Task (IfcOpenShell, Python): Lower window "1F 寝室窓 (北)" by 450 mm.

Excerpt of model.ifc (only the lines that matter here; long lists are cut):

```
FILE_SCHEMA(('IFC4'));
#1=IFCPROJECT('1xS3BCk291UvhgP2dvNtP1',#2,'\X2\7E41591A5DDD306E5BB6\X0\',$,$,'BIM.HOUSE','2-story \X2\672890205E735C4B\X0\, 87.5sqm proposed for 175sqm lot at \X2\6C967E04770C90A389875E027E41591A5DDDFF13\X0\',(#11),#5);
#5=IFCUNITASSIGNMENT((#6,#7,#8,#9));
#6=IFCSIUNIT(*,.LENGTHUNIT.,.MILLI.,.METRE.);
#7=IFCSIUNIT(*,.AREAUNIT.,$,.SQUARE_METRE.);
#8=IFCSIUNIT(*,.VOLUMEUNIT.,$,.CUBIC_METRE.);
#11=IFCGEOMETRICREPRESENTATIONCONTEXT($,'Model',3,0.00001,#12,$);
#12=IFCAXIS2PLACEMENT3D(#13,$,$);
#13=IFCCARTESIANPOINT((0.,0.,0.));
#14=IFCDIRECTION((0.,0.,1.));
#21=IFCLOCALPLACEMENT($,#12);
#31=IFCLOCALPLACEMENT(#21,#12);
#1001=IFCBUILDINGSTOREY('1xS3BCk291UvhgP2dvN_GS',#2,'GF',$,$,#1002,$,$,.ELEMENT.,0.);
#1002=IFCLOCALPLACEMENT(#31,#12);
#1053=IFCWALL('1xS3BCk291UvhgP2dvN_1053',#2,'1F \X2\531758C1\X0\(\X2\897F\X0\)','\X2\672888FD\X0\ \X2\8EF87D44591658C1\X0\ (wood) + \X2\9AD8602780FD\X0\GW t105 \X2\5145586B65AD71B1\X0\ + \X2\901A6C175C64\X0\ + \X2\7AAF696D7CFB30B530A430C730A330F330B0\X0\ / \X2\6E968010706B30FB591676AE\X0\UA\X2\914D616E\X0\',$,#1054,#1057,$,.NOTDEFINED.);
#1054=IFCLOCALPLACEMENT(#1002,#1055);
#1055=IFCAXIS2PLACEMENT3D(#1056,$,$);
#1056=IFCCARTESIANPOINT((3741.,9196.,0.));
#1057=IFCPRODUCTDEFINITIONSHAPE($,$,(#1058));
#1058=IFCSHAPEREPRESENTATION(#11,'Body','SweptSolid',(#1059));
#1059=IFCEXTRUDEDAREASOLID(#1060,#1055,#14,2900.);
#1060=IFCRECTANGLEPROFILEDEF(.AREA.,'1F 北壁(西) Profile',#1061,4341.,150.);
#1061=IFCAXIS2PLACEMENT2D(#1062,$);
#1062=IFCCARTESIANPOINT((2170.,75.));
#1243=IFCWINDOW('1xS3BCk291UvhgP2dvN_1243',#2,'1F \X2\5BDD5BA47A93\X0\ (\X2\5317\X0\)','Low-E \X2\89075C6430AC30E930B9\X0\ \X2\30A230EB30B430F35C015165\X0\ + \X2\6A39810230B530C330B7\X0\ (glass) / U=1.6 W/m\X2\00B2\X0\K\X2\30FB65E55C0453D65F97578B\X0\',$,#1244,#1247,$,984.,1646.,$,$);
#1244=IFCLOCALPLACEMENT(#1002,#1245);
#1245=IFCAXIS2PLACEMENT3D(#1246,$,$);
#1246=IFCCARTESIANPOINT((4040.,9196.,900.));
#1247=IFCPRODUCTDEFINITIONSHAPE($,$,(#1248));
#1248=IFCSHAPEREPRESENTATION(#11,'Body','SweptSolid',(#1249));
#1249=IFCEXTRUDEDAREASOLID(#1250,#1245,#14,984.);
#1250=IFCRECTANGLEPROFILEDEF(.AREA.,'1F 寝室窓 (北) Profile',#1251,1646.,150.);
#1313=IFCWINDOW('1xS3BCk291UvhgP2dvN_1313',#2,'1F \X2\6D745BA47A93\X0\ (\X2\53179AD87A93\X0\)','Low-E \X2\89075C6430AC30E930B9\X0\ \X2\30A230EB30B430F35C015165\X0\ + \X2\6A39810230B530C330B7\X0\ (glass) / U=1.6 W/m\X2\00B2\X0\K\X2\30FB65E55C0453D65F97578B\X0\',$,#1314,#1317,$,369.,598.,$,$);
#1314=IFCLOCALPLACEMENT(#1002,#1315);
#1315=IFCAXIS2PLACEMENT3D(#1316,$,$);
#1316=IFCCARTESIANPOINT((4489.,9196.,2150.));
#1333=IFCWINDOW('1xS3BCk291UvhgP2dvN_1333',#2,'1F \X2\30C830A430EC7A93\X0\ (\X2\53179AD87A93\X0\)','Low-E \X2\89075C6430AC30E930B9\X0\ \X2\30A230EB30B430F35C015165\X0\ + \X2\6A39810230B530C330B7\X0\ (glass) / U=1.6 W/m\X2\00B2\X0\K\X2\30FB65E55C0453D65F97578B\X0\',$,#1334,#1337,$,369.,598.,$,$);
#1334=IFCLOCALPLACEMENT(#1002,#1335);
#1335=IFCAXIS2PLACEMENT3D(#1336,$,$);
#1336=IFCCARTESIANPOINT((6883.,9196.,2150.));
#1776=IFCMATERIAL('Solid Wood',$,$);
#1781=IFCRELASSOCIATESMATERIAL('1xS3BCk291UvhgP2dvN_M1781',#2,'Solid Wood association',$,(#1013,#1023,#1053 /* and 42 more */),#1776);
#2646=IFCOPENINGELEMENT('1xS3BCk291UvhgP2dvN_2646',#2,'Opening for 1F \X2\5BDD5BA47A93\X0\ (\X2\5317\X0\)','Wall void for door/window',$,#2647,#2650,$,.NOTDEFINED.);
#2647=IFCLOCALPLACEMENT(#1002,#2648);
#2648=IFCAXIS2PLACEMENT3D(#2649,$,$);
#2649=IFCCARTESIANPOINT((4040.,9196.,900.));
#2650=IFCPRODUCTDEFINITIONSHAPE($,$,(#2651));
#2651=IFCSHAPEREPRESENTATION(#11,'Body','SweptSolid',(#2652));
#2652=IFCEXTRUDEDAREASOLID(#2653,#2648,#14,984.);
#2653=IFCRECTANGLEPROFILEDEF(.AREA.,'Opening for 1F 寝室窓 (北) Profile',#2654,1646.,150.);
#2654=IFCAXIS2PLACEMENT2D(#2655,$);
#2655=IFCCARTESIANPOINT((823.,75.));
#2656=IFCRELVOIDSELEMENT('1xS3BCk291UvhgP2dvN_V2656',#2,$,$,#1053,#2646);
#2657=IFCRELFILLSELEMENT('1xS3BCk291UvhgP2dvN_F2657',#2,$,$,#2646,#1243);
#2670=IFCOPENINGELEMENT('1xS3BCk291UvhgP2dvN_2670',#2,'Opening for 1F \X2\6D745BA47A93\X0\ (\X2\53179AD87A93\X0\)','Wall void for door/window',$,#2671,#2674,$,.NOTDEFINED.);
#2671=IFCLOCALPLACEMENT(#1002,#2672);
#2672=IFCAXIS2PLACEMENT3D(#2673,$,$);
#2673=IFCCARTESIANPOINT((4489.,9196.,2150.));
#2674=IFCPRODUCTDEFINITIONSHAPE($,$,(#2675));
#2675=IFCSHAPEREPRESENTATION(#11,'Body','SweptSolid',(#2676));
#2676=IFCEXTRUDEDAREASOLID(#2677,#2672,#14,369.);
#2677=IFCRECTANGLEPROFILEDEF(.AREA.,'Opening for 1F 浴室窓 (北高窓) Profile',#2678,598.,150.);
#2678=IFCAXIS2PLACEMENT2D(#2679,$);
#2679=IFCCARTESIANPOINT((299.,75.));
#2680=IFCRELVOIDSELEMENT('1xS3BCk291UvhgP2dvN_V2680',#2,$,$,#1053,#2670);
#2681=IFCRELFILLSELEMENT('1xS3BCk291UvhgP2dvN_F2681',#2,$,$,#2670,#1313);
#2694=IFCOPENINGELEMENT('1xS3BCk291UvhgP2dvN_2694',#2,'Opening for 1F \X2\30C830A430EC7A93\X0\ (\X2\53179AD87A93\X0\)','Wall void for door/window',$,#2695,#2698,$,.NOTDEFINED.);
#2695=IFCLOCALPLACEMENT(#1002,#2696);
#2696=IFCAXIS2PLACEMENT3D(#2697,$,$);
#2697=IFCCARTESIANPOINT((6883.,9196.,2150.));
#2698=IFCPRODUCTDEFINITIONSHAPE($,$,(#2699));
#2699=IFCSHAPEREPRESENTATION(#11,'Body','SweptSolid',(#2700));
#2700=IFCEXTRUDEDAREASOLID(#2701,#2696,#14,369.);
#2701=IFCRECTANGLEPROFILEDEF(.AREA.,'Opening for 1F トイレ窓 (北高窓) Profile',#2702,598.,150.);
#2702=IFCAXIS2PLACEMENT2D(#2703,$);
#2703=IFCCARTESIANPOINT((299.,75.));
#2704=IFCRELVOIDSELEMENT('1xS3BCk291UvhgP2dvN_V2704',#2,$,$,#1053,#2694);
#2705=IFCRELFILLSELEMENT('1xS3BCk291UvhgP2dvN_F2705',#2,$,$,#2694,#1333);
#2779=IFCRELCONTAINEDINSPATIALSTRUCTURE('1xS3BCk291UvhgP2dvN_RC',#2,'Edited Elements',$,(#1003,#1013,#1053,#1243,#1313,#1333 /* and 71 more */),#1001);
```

```python
import numpy as np
import ifcopenshell
import ifcopenshell.api.geometry
import ifcopenshell.util.placement
import ifcopenshell.util.unit

model = ifcopenshell.open("model.ifc")
unit_scale = ifcopenshell.util.unit.calculate_unit_scale(model)

window = model.by_guid("1xS3BCk291UvhgP2dvN_1243")
opening = window.FillsVoids[0].RelatingOpeningElement
dz = -450.0

shift = np.array([0.0, 0.0, dz])
# The window is not placed relative to its opening, so move both.
for product in (opening, window):
    matrix = ifcopenshell.util.placement.get_local_placement(product.ObjectPlacement)
    matrix[:3, 3] += shift
    ifcopenshell.api.geometry.edit_object_placement(model, product=product, matrix=matrix, is_si=False)

print(f"moved by {dz * unit_scale:+.3f} m")

model.write("model_v2.ifc")
```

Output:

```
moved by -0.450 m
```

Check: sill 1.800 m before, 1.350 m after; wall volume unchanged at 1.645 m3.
